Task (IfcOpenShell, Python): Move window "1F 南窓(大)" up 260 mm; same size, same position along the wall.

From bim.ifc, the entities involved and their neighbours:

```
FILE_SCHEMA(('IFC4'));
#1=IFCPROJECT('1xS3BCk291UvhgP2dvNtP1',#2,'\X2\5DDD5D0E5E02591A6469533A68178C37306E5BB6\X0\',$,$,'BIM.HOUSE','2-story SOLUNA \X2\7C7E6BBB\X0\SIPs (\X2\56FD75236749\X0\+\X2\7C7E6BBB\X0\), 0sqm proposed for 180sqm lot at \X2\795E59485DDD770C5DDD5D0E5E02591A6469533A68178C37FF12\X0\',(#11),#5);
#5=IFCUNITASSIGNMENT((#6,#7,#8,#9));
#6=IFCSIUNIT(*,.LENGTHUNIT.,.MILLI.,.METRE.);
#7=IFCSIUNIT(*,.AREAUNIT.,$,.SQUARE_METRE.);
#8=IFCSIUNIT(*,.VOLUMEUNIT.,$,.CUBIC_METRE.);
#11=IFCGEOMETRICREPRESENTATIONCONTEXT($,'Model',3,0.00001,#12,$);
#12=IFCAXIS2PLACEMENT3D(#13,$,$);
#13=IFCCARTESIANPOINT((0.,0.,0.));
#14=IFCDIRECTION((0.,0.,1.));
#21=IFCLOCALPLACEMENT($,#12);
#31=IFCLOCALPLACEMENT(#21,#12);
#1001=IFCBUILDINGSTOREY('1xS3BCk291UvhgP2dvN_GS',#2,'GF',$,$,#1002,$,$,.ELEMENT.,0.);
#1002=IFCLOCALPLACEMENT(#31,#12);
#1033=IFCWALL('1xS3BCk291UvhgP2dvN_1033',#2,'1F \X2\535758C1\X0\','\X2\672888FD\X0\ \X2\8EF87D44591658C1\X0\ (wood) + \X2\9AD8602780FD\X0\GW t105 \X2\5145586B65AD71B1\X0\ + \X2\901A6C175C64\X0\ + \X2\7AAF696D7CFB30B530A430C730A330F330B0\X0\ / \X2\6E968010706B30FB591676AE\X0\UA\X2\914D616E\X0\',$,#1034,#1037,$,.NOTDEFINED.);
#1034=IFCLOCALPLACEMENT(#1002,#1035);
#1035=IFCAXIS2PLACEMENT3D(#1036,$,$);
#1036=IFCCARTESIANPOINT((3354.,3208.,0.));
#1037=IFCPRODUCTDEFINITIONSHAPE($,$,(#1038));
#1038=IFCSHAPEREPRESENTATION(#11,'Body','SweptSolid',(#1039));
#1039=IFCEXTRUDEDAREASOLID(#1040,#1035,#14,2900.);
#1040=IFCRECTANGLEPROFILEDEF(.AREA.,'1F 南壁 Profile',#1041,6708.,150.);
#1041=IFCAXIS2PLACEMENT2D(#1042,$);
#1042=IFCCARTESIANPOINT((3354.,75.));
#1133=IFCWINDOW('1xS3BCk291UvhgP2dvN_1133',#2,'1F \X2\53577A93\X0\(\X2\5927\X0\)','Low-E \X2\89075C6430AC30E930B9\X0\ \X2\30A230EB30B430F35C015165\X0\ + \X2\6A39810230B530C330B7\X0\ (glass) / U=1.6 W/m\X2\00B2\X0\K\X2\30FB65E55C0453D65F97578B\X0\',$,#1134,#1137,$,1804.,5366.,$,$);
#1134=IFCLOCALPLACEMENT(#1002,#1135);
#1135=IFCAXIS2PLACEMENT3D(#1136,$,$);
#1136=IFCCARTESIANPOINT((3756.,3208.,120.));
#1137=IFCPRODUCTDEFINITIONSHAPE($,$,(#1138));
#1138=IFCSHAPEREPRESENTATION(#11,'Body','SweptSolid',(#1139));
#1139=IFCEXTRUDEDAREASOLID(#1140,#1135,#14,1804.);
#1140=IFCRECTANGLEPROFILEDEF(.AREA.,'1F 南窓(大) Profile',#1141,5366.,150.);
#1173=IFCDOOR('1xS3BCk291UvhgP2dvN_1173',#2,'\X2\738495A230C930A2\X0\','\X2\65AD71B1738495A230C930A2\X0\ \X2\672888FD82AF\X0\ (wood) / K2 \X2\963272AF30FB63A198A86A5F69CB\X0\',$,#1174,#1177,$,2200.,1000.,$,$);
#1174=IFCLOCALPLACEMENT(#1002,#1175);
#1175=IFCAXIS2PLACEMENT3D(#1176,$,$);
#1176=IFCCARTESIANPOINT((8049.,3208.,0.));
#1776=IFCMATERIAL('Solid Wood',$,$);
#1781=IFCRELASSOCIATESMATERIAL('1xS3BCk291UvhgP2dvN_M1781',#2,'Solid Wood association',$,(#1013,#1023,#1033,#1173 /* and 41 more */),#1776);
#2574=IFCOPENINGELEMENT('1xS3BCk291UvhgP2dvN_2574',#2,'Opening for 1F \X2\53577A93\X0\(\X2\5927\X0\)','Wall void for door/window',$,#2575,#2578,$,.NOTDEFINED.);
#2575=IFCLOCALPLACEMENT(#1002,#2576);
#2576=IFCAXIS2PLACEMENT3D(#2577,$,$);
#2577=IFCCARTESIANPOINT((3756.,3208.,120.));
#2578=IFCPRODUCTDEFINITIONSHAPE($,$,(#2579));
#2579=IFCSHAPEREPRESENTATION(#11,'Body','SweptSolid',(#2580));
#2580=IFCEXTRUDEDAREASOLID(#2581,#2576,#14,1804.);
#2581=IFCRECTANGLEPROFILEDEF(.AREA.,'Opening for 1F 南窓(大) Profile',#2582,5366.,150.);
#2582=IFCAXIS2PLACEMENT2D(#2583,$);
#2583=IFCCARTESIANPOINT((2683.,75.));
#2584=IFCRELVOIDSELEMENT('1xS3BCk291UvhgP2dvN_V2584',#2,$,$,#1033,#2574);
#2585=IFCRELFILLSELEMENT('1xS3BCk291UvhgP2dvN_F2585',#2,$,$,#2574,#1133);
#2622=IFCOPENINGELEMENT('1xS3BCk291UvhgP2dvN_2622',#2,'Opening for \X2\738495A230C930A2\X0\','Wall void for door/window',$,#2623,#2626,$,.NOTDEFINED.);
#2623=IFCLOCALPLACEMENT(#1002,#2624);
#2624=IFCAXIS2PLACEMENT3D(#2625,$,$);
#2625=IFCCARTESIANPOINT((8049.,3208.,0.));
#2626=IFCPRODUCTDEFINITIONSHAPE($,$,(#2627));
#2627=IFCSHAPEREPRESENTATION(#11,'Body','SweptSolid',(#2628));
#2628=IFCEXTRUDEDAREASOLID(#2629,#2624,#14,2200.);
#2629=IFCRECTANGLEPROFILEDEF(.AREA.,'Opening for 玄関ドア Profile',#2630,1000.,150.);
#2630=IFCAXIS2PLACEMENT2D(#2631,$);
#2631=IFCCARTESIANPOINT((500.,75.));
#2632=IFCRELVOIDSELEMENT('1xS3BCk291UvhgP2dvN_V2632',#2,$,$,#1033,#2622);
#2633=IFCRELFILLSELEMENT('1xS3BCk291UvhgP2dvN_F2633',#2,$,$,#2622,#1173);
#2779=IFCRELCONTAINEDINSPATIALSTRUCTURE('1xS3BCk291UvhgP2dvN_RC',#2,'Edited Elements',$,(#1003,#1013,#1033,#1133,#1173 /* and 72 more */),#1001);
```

```python
import numpy as np
import ifcopenshell
import ifcopenshell.api.geometry
import ifcopenshell.util.placement
import ifcopenshell.util.unit

model = ifcopenshell.open("bim.ifc")
unit_scale = ifcopenshell.util.unit.calculate_unit_scale(model)

window = model.by_guid("1xS3BCk291UvhgP2dvN_1133")
opening = window.FillsVoids[0].RelatingOpeningElement
dz = 0.26 / unit_scale

shift = np.array([0.0, 0.0, dz])
# The window is not placed relative to its opening, so move both.
for product in (opening, window):
    matrix = ifcopenshell.util.placement.get_local_placement(product.ObjectPlacement)
    matrix[:3, 3] += shift
    ifcopenshell.api.geometry.edit_object_placement(model, product=product, matrix=matrix, is_si=False)

print(f"moved by {dz * unit_scale:+.3f} m")

model.write("bim_edited.ifc")
```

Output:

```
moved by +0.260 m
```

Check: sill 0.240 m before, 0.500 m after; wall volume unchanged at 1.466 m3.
